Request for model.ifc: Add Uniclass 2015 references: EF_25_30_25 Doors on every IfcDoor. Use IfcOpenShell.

First a look at what the model holds.

```python
import ifcopenshell

model = ifcopenshell.open("model.ifc")
print(model.schema)
print("classifications:", [c.Name for c in model.by_type("IfcClassification")])
for ifc_class in ("IfcDoor", "IfcRoof", "IfcStair", "IfcWall", "IfcWindow"):
    print(ifc_class, len(model.by_type(ifc_class)))
```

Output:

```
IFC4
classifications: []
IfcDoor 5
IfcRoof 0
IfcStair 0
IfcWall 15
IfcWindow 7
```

```python
import ifcopenshell
import ifcopenshell.api.classification

model = ifcopenshell.open("model.ifc")

system = ifcopenshell.api.classification.add_classification(model, classification="Uniclass 2015")

codes = {
    "IfcDoor": ("EF_25_30_25", "Doors"),
}
for ifc_class, (code, name) in codes.items():
    products = model.by_type(ifc_class)
    ifcopenshell.api.classification.add_reference(
        model, products=products, classification=system, identification=code, name=name
    )
    print(code, len(products))

model.write("model_edited.ifc")
```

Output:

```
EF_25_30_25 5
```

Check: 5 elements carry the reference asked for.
